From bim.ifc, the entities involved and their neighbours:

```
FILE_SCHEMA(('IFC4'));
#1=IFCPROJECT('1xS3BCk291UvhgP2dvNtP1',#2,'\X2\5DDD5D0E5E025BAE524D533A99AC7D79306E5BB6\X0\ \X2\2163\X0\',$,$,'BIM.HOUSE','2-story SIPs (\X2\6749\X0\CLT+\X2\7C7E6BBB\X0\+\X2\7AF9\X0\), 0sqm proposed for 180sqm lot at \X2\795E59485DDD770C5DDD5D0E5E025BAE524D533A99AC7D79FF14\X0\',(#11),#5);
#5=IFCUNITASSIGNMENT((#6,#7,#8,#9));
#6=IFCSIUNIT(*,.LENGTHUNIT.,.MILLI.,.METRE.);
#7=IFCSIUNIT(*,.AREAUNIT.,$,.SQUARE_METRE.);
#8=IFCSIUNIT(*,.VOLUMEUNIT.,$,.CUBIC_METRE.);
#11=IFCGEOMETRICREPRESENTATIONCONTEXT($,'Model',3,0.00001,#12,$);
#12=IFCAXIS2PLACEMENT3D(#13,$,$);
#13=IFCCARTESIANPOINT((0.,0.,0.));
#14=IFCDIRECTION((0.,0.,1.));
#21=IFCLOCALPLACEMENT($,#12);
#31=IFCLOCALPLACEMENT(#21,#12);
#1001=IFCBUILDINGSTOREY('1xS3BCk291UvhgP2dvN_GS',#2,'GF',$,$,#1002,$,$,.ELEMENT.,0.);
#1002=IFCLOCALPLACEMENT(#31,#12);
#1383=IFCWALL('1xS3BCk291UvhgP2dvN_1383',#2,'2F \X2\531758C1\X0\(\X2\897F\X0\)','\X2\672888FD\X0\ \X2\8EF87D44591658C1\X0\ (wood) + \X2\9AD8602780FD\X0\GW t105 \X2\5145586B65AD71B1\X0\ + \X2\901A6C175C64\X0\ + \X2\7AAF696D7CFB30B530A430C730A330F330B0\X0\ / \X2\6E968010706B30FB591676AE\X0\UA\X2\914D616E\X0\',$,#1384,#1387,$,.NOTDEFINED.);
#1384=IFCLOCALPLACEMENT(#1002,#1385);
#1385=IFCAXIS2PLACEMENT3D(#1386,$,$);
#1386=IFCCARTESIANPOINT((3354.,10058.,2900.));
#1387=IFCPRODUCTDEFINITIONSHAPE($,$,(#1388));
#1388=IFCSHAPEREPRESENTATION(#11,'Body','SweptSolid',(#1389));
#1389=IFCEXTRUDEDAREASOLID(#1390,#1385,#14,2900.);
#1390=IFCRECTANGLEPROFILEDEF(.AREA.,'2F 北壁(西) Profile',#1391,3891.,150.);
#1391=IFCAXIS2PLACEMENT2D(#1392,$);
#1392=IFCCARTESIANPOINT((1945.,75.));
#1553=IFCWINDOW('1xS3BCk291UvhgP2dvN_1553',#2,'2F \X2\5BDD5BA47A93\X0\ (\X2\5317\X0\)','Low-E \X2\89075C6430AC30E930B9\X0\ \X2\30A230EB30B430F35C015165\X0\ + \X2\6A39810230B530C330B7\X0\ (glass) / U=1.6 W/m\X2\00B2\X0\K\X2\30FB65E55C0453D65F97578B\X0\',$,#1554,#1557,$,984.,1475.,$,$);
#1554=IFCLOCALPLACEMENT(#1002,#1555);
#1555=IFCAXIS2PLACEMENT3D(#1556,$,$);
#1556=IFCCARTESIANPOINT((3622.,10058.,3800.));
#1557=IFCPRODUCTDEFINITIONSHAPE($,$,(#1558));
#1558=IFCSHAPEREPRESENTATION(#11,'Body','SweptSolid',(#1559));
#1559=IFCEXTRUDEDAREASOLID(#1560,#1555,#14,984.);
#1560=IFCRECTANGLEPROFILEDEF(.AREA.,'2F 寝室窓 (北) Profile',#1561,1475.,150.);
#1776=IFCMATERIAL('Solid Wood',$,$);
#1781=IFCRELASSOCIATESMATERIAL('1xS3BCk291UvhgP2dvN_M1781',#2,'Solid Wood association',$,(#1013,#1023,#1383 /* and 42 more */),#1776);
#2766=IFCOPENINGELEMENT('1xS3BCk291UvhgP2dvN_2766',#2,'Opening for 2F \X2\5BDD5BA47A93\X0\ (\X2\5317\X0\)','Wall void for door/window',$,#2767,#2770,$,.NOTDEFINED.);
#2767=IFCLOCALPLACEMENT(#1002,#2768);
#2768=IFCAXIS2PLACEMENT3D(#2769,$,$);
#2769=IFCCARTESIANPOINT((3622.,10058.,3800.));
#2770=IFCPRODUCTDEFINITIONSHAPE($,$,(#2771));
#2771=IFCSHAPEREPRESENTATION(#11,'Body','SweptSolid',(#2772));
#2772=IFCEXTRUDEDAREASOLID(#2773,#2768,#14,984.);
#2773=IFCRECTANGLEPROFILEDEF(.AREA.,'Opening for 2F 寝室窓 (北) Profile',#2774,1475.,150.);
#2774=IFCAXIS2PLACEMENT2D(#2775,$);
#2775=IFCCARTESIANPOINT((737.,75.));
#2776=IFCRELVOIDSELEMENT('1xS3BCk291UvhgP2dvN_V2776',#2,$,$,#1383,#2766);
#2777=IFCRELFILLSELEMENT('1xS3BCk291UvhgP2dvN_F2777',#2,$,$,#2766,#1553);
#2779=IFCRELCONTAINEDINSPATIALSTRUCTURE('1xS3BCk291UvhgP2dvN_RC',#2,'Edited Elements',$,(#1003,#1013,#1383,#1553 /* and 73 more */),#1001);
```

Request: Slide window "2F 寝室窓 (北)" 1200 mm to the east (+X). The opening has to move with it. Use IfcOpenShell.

```python
import ifcopenshell
import ifcopenshell.api.geometry
import ifcopenshell.util.placement
import ifcopenshell.util.unit

model = ifcopenshell.open("bim.ifc")
unit_scale = ifcopenshell.util.unit.calculate_unit_scale(model)

window = model.by_guid("1xS3BCk291UvhgP2dvN_1553")
opening = window.FillsVoids[0].RelatingOpeningElement
wall = opening.VoidsElements[0].RelatingBuildingElement

wall_matrix = ifcopenshell.util.placement.get_local_placement(wall.ObjectPlacement)
shift = wall_matrix[:3, 0] * 1.2 / unit_scale
before = ifcopenshell.util.placement.get_local_placement(window.ObjectPlacement)[:3, 3].copy()

# The window is not placed relative to its opening, so move both.
for product in (opening, window):
    matrix = ifcopenshell.util.placement.get_local_placement(product.ObjectPlacement)
    matrix[:3, 3] += shift
    ifcopenshell.api.geometry.edit_object_placement(model, product=product, matrix=matrix, is_si=False)

after = ifcopenshell.util.placement.get_local_placement(window.ObjectPlacement)[:3, 3]
print("window moved by", (after - before).round(3) + 0.0)

model.write("bim_rev.ifc")
```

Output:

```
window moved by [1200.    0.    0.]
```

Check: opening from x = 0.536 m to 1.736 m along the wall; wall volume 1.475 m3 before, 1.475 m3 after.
